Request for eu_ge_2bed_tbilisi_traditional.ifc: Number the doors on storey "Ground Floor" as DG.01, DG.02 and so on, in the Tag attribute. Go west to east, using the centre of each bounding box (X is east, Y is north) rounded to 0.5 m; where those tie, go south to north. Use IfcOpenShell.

First a look at what the model holds.

```python
import ifcopenshell
import ifcopenshell.util.element
import ifcopenshell.util.placement

model = ifcopenshell.open("eu_ge_2bed_tbilisi_traditional.ifc")
print(model.schema)
storey = next(s for s in model.by_type("IfcBuildingStorey") if s.Name == "Ground Floor")
doors = [e for e in ifcopenshell.util.element.get_decomposition(storey) if e.is_a("IfcDoor")]
for e in sorted(doors, key=lambda e: e.id()):
    origin = ifcopenshell.util.placement.get_local_placement(e.ObjectPlacement)[:3, 3]
    print(e.id(), e.Tag, e.Name, origin.round(2) + 0.0, sep=" | ")
```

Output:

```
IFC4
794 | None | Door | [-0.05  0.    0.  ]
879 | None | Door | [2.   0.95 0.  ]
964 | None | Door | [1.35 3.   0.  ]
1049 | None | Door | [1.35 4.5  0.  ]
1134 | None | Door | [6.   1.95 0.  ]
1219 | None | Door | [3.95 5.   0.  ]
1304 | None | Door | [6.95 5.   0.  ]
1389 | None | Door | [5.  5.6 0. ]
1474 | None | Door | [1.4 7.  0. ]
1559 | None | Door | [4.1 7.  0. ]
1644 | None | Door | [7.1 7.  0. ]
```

```python
import ifcopenshell
import ifcopenshell.geom
import ifcopenshell.util.element
import ifcopenshell.util.shape

model = ifcopenshell.open("eu_ge_2bed_tbilisi_traditional.ifc")
settings = ifcopenshell.geom.settings()
settings.set("use-world-coords", True)


def centre(element):
    shape = ifcopenshell.geom.create_shape(settings, element)
    return ifcopenshell.util.shape.get_bbox_centroid(shape.geometry)


storey = next(s for s in model.by_type("IfcBuildingStorey") if s.Name == "Ground Floor")
doors = [e for e in ifcopenshell.util.element.get_decomposition(storey) if e.is_a("IfcDoor")]

# Insertion points can sit at a corner or the storey origin, so sort by the geometry (in metres).
centres = {e: centre(e) for e in doors}
doors.sort(key=lambda e: (round(centres[e][0] / 0.5), centres[e][1]))

for i, e in enumerate(doors, start=1):
    number = f"DG.{i:02d}"
    e.Tag = number
    print(e.id(), number)

model.write("eu_ge_2bed_tbilisi_traditional_v2.ifc")
```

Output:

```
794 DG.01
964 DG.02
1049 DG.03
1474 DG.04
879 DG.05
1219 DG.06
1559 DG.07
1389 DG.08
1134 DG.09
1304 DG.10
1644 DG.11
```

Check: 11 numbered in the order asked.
